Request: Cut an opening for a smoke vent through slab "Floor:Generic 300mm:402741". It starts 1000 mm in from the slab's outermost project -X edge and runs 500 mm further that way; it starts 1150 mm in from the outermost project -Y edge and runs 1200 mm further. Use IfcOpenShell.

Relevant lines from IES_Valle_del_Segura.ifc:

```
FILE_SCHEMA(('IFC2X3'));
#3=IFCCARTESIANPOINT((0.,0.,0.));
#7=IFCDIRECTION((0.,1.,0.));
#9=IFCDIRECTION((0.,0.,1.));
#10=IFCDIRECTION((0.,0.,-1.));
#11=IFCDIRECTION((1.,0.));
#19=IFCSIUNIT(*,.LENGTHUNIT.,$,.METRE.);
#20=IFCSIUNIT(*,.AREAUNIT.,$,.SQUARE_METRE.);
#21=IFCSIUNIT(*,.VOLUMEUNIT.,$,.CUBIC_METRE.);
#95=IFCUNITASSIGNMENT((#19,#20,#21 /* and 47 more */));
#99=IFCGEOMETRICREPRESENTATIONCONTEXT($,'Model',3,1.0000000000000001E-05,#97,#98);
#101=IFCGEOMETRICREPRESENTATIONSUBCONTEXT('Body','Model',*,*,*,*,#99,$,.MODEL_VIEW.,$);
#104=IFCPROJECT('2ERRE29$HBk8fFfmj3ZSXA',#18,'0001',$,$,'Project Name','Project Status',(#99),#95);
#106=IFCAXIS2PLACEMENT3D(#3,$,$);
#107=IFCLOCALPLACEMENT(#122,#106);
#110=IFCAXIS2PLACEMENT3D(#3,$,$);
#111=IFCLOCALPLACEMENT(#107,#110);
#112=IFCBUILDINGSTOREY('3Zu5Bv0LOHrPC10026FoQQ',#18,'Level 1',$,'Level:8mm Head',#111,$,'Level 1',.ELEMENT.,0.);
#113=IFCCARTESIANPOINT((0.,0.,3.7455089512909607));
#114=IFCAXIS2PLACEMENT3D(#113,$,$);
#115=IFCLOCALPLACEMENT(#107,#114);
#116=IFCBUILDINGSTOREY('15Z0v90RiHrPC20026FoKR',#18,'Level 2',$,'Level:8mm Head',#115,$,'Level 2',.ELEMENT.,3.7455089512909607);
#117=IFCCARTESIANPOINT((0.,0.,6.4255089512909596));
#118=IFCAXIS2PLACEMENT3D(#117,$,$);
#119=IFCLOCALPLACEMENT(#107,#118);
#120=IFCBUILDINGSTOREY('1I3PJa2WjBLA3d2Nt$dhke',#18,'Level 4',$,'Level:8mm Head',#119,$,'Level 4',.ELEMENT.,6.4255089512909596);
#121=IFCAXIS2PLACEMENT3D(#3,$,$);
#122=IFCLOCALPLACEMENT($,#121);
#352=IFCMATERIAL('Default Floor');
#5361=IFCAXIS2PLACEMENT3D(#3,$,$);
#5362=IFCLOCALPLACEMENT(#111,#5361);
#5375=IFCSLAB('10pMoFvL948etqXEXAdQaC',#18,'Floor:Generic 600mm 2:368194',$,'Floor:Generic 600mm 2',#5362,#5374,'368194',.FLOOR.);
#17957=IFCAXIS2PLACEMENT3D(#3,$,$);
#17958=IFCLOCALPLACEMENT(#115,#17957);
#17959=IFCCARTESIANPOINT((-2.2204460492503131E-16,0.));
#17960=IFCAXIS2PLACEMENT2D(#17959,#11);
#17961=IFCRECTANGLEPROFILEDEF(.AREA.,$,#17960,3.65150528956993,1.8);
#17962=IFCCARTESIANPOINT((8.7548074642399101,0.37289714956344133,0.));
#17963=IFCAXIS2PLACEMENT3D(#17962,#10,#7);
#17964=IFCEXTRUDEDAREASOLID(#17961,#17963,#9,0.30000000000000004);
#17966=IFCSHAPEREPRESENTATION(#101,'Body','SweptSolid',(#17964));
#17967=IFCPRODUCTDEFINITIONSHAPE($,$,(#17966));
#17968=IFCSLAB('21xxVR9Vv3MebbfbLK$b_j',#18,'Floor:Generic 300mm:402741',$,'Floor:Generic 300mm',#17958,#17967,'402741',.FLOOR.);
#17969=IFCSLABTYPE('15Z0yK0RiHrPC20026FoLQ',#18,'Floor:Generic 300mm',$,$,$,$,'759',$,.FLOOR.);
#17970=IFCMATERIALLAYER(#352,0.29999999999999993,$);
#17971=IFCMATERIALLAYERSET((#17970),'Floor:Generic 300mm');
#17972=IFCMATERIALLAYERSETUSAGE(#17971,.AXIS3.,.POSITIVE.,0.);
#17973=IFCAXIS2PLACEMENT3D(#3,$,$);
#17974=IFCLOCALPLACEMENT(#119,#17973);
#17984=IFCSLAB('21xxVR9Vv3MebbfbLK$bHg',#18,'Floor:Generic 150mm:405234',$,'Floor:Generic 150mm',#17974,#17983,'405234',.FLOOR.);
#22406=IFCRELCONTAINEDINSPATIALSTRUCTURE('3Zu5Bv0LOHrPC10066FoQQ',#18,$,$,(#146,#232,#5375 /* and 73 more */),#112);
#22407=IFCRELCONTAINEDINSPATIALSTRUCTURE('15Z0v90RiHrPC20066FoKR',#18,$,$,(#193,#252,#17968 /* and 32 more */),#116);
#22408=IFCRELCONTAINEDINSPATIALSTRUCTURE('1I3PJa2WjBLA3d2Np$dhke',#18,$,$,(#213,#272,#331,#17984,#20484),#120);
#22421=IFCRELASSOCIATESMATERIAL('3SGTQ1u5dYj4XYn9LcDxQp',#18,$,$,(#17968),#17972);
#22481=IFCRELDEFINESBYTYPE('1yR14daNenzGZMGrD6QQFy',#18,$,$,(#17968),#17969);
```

```python
import numpy as np
import ifcopenshell
import ifcopenshell.api.feature
import ifcopenshell.api.geometry
import ifcopenshell.api.root
import ifcopenshell.geom
import ifcopenshell.util.placement
import ifcopenshell.util.representation
import ifcopenshell.util.shape
import ifcopenshell.util.unit

model = ifcopenshell.open("IES_Valle_del_Segura.ifc")
unit_scale = ifcopenshell.util.unit.calculate_unit_scale(model)
settings = ifcopenshell.geom.settings()


def volume(element):
    """Net volume in cubic metres, openings subtracted."""
    shape = ifcopenshell.geom.create_shape(settings, element)
    return ifcopenshell.util.shape.get_volume(shape.geometry)


slab = model.by_guid("21xxVR9Vv3MebbfbLK$b_j")
before = volume(slab)

# Extent in the slab's own axes, in metres. The edges named are its -X and -Y sides.
slab_shape = ifcopenshell.geom.create_shape(settings, slab)
vertices = ifcopenshell.util.shape.get_vertices(slab_shape.geometry)
x_min, y_min, bottom = vertices.min(axis=0)
top = vertices[:, 2].max()

opening = ifcopenshell.api.root.create_entity(model, ifc_class="IfcOpeningElement", name="Smoke vent opening")
context = ifcopenshell.util.representation.get_context(model, "Model", "Body", "MODEL_VIEW")
width, depth = 0.5, 1.2
outline = [(0.0, 0.0), (width, 0.0), (width, depth), (0.0, depth), (0.0, 0.0)]
# Overshoot both faces by 50 mm so the cut is clean.
shape = ifcopenshell.api.geometry.add_slab_representation(
    model, context=context, depth=top - bottom + 0.1, polyline=outline
)
ifcopenshell.api.geometry.assign_representation(model, product=opening, representation=shape)

matrix = ifcopenshell.util.placement.get_local_placement(slab.ObjectPlacement)
matrix[:, 3] = matrix @ np.append(np.array([x_min + 1, y_min + 1.15, bottom - 0.05]) / unit_scale, 1.0)
ifcopenshell.api.geometry.edit_object_placement(model, product=opening, matrix=matrix, is_si=False)
ifcopenshell.api.feature.add_feature(model, feature=opening, element=slab)

after = volume(slab)

print(f"slab volume {before:.3f} -> {after:.3f} m3")

model.write("IES_Valle_del_Segura-out.ifc")
```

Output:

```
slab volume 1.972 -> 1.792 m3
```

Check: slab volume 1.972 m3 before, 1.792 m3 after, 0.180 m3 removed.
